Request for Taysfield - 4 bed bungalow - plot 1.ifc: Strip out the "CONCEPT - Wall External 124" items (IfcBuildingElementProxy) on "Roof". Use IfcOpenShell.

First a look at what the model holds.

```python
import ifcopenshell
import ifcopenshell.util.element

model = ifcopenshell.open("Taysfield - 4 bed bungalow - plot 1.ifc")
print(model.schema)
storey = next(s for s in model.by_type("IfcBuildingStorey") if s.Name == "Roof")
proxies = [e for e in ifcopenshell.util.element.get_decomposition(storey) if e.is_a("IfcBuildingElementProxy")]
seen = {}
for e in proxies:
    element_type = ifcopenshell.util.element.get_type(e)
    name = element_type.Name if element_type not in (None, e) else None
    seen[name] = seen.get(name, 0) + 1
for name, count in sorted(seen.items(), key=str):
    print(count, "x", name)
```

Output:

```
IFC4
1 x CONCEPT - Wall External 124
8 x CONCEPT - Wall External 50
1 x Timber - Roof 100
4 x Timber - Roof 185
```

```python
import ifcopenshell
import ifcopenshell.api.root
import ifcopenshell.util.element

model = ifcopenshell.open("Taysfield - 4 bed bungalow - plot 1.ifc")

storey = next(s for s in model.by_type("IfcBuildingStorey") if s.Name == "Roof")
proxies = [e for e in ifcopenshell.util.element.get_decomposition(storey) if e.is_a("IfcBuildingElementProxy")]
targets = [e for e in proxies if (t := ifcopenshell.util.element.get_type(e)) not in (None, e) and t.Name == "CONCEPT - Wall External 124"]

for e in targets:
    ifcopenshell.api.root.remove_product(model, product=e)
print(len(targets), "removed")

model.write("Taysfield - 4 bed bungalow - plot 1_rev.ifc")
```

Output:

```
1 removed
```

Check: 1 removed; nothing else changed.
